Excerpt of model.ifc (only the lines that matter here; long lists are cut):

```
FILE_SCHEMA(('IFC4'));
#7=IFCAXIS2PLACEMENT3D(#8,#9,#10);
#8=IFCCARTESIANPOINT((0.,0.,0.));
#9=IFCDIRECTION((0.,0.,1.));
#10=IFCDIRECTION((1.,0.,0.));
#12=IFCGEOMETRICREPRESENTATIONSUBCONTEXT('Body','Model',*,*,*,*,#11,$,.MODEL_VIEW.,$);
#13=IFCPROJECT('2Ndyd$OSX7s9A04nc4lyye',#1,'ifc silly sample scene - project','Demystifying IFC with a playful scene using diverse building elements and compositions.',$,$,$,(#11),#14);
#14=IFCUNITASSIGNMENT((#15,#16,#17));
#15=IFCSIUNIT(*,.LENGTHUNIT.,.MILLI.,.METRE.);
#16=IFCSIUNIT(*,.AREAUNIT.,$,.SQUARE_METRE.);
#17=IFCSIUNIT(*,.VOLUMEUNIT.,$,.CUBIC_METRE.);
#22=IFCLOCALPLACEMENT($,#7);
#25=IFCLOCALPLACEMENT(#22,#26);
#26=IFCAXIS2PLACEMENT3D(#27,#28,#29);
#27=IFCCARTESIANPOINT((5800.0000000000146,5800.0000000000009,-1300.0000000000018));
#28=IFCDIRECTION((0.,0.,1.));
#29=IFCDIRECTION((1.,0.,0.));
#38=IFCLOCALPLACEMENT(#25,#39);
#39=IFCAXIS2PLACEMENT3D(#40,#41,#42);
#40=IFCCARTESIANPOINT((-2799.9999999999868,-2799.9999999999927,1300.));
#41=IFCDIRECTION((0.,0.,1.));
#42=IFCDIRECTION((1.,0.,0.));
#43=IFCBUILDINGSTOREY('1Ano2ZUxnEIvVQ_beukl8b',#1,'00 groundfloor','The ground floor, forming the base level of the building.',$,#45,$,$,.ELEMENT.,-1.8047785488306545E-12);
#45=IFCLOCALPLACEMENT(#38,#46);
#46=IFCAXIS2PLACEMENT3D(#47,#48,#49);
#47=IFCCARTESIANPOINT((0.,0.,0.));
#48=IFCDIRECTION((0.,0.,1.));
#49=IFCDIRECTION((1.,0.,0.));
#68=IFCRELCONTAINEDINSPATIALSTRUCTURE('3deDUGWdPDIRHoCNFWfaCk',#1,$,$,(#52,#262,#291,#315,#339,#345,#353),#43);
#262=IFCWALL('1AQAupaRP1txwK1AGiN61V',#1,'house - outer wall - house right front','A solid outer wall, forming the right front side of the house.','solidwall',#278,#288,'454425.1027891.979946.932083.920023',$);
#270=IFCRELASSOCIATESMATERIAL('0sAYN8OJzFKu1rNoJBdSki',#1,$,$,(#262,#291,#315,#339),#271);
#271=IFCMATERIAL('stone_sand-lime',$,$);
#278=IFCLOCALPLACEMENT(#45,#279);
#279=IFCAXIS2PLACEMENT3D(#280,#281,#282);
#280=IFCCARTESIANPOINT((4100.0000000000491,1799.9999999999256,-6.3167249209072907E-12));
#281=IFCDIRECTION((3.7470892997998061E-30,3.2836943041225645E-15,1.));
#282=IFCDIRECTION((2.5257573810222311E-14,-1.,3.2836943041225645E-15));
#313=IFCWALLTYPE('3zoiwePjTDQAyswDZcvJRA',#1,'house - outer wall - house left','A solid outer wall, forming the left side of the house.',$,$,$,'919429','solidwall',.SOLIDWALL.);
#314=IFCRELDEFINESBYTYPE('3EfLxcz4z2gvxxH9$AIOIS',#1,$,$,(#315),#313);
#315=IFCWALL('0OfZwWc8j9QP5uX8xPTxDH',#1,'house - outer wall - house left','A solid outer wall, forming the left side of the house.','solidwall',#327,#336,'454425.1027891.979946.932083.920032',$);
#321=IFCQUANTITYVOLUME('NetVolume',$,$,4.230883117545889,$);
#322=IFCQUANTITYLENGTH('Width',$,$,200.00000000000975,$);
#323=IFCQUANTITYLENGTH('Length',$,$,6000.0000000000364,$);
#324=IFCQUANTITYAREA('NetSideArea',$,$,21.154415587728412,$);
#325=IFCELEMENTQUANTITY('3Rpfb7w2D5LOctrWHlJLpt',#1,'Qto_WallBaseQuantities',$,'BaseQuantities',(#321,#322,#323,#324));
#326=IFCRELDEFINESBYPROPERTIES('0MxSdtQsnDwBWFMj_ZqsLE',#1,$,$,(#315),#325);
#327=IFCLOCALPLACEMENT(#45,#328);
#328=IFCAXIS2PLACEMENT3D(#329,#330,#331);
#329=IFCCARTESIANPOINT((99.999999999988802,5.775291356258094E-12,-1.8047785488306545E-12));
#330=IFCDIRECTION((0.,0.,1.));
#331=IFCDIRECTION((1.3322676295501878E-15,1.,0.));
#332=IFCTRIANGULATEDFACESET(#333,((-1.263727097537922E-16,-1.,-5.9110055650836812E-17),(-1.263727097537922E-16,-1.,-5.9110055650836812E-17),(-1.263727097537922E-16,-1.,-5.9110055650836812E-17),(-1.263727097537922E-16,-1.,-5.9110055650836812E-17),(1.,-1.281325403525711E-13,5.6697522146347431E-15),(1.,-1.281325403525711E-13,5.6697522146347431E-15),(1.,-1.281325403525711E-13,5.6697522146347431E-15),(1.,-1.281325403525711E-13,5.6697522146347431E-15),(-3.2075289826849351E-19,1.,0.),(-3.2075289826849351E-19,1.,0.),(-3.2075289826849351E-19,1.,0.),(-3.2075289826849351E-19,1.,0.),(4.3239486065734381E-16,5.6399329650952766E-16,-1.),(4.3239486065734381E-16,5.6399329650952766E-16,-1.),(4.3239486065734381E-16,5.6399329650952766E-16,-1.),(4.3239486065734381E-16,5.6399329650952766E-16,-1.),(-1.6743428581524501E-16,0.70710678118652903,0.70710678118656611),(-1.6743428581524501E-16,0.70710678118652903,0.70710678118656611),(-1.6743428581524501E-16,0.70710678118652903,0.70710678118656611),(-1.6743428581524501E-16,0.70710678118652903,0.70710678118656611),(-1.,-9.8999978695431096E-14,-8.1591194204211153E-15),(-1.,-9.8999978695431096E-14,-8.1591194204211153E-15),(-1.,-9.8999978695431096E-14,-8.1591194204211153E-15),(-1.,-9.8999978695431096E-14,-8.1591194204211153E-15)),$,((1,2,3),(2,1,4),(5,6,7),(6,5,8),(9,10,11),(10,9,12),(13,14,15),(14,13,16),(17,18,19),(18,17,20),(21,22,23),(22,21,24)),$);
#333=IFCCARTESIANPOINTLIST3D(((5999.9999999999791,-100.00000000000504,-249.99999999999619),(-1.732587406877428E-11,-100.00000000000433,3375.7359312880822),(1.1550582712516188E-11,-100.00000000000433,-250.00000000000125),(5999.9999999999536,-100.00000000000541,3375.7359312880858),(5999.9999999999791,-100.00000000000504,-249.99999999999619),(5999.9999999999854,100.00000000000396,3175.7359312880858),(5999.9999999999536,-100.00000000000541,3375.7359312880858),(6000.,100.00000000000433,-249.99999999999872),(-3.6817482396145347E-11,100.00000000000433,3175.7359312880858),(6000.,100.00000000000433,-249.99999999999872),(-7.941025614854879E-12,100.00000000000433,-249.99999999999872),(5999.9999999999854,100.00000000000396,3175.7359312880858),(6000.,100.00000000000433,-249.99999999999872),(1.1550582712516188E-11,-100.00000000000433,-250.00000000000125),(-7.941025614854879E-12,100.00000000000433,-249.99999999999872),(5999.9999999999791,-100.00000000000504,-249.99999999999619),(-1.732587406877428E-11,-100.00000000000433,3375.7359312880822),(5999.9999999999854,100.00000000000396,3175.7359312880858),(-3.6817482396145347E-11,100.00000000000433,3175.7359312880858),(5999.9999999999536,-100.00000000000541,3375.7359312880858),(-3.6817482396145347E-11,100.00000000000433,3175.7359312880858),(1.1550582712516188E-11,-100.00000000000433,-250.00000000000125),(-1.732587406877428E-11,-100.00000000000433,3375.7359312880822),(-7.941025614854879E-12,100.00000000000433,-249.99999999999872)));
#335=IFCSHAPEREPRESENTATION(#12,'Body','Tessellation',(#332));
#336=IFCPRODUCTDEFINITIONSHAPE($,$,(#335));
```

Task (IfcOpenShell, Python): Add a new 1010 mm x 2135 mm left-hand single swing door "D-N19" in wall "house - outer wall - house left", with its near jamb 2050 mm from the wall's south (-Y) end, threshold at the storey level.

```python
import numpy as np
import ifcopenshell
import ifcopenshell.api.feature
import ifcopenshell.api.geometry
import ifcopenshell.api.pset
import ifcopenshell.api.root
import ifcopenshell.api.spatial
import ifcopenshell.geom
import ifcopenshell.util.element
import ifcopenshell.util.placement
import ifcopenshell.util.representation
import ifcopenshell.util.shape
import ifcopenshell.util.unit

model = ifcopenshell.open("model.ifc")
unit_scale = ifcopenshell.util.unit.calculate_unit_scale(model)
area_scale = ifcopenshell.util.unit.calculate_unit_scale(model, "AREAUNIT")
volume_scale = ifcopenshell.util.unit.calculate_unit_scale(model, "VOLUMEUNIT")
settings = ifcopenshell.geom.settings()


def volume(element):
    """Net volume in cubic metres, openings subtracted."""
    shape = ifcopenshell.geom.create_shape(settings, element)
    return ifcopenshell.util.shape.get_volume(shape.geometry)


wall = model.by_guid("0OfZwWc8j9QP5uX8xPTxDH")
storey = ifcopenshell.util.element.get_container(wall, ifc_class="IfcBuildingStorey")
context = ifcopenshell.util.representation.get_context(model, "Model", "Body", "MODEL_VIEW")
before = volume(wall)

width, height, from_end, sill = 1.01, 2.135, 2.05, 0.0  # metres

# The wall runs along its own X axis, and the end named is its -X end.
wall_shape = ifcopenshell.geom.create_shape(settings, wall)
x, y, z = ifcopenshell.util.shape.get_vertices(wall_shape.geometry).T
start = x.min() + from_end
face, thickness = float(y.min()), float(y.max() - y.min())
wall_matrix = ifcopenshell.util.placement.get_local_placement(wall.ObjectPlacement)
level = ifcopenshell.util.placement.get_local_placement(storey.ObjectPlacement)[2, 3]


def in_wall(x, y):
    """Placement at x, y metres in the wall's axes, at sill height."""
    matrix = wall_matrix.copy()
    matrix[:, 3] = wall_matrix @ np.array([x / unit_scale, y / unit_scale, 0.0, 1.0])
    matrix[2, 3] = level + sill / unit_scale
    return matrix


# Opening: a box that overshoots both wall faces by 50 mm.
opening = ifcopenshell.api.root.create_entity(model, ifc_class="IfcOpeningElement", predefined_type="OPENING")
box = ifcopenshell.api.geometry.add_wall_representation(
    model, context=context, length=width, height=height, thickness=thickness + 0.1
)
ifcopenshell.api.geometry.assign_representation(model, product=opening, representation=box)
ifcopenshell.api.geometry.edit_object_placement(model, product=opening, matrix=in_wall(start, face - 0.05), is_si=False)
ifcopenshell.api.feature.add_feature(model, feature=opening, element=wall)

door = ifcopenshell.api.root.create_entity(model, ifc_class="IfcDoor", name="D-N19", predefined_type="DOOR")
door.OverallWidth, door.OverallHeight = width / unit_scale, height / unit_scale
door.OperationType = "SINGLE_SWING_LEFT"
body = ifcopenshell.api.geometry.add_door_representation(
    model,
    context=context,
    overall_width=door.OverallWidth,
    overall_height=door.OverallHeight,
    operation_type="SINGLE_SWING_LEFT",
    lining_properties={"LiningDepth": thickness / unit_scale, "ThresholdDepth": thickness / unit_scale},
)
ifcopenshell.api.geometry.assign_representation(model, product=door, representation=body)
ifcopenshell.api.spatial.assign_container(model, products=[door], relating_structure=storey)
ifcopenshell.api.feature.add_filling(model, opening=opening, element=door)

# The lining spans the wall, so the door starts at the wall face.
ifcopenshell.api.geometry.edit_object_placement(model, product=door, matrix=in_wall(start, face), is_si=False)

after = volume(wall)

# Update the wall's stored quantities.
qto = model.by_id(ifcopenshell.util.element.get_pset(wall, "Qto_WallBaseQuantities", should_inherit=False)["id"])
ifcopenshell.api.pset.edit_qto(model, qto=qto, properties={
    "NetVolume": after / volume_scale,
    "NetSideArea": after / thickness / area_scale,
})

print(f"wall volume {before:.3f} -> {after:.3f} m3")

model.write("model_updated.ifc")
```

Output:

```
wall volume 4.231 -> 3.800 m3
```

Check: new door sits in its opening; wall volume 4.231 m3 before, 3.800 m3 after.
